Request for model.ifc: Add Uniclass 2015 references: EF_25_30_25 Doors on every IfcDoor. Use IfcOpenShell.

First a look at what the model holds.

```python
import ifcopenshell

model = ifcopenshell.open("model.ifc")
print(model.schema)
print("classifications:", [c.Name for c in model.by_type("IfcClassification")])
for ifc_class in ("IfcDoor", "IfcRoof", "IfcStair", "IfcWall", "IfcWindow"):
    print(ifc_class, len(model.by_type(ifc_class)))
```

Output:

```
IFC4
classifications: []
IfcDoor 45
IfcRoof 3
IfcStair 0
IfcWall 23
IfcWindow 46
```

```python
import ifcopenshell
import ifcopenshell.api.classification

model = ifcopenshell.open("model.ifc")

system = ifcopenshell.api.classification.add_classification(model, classification="Uniclass 2015")

codes = {
    "IfcDoor": ("EF_25_30_25", "Doors"),
}
for ifc_class, (code, name) in codes.items():
    products = model.by_type(ifc_class)
    ifcopenshell.api.classification.add_reference(
        model, products=products, classification=system, identification=code, name=name
    )
    print(code, len(products))

model.write("model_rev.ifc")
```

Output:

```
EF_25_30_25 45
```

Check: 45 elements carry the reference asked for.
